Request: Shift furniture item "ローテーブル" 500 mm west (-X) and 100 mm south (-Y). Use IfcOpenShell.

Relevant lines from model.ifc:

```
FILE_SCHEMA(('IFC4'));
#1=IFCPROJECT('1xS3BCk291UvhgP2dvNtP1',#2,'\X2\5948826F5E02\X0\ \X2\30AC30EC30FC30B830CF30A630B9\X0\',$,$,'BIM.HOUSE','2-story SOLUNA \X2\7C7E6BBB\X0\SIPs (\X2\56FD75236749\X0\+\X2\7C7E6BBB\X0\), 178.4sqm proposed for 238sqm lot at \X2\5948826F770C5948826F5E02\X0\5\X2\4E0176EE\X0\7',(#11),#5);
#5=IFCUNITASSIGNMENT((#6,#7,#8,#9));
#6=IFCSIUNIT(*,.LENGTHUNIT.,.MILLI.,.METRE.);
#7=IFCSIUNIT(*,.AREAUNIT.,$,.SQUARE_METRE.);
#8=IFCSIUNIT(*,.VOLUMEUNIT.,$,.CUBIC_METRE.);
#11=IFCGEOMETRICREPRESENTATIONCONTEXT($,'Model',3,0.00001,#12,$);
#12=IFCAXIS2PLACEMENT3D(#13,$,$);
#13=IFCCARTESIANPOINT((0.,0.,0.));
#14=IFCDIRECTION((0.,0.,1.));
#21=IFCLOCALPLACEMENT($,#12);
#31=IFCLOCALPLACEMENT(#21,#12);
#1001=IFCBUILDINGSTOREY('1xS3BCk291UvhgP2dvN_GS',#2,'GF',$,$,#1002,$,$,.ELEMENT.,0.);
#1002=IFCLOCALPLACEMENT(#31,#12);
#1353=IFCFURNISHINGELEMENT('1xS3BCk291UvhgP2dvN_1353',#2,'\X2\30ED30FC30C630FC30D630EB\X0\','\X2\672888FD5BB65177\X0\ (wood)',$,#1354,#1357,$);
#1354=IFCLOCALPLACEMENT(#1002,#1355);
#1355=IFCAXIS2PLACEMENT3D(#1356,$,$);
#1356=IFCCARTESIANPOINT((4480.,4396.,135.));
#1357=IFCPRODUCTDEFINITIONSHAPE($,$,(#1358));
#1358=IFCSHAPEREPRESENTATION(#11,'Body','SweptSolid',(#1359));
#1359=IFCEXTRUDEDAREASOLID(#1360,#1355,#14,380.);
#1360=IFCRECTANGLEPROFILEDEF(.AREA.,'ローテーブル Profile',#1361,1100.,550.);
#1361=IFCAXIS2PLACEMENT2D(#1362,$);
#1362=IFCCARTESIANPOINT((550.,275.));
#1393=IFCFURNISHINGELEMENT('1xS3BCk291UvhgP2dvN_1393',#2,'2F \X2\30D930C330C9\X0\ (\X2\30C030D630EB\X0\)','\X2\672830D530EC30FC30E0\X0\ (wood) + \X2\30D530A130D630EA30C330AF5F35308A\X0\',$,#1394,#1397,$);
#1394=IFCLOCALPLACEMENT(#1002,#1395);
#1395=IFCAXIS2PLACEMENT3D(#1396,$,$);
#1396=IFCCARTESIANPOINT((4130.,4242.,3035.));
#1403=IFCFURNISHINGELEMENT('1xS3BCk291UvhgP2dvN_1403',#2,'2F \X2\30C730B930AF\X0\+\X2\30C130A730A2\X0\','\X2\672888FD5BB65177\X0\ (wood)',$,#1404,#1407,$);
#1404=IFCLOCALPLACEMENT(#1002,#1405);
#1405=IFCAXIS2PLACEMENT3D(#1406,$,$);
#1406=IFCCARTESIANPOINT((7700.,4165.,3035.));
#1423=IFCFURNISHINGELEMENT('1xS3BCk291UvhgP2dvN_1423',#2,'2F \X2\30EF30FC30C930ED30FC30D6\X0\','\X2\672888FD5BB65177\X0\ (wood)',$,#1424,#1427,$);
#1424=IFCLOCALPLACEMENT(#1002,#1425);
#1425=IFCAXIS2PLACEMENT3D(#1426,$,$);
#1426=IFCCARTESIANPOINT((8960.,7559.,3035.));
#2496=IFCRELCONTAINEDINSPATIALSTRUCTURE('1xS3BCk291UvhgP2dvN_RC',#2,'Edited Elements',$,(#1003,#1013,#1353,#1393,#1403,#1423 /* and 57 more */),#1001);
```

```python
import ifcopenshell
import ifcopenshell.api.geometry
import ifcopenshell.util.placement

model = ifcopenshell.open("model.ifc")

item = model.by_guid("1xS3BCk291UvhgP2dvN_1353")
matrix = ifcopenshell.util.placement.get_local_placement(item.ObjectPlacement)
matrix[0, 3] -= 500.0
matrix[1, 3] -= 100.0
ifcopenshell.api.geometry.edit_object_placement(model, product=item, matrix=matrix, is_si=False)

print(ifcopenshell.util.placement.get_local_placement(item.ObjectPlacement).round(3) + 0.0)

model.write("model_rev.ifc")
```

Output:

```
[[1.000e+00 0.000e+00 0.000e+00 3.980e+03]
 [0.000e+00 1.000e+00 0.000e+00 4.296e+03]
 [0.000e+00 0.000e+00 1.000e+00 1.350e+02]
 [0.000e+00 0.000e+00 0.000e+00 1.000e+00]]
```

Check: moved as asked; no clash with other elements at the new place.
